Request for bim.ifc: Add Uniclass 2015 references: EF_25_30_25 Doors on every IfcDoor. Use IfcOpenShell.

First a look at what the model holds.

```python
import ifcopenshell

model = ifcopenshell.open("bim.ifc")
print(model.schema)
print("classifications:", [c.Name for c in model.by_type("IfcClassification")])
for ifc_class in ("IfcDoor", "IfcRoof", "IfcStair", "IfcWall", "IfcWindow"):
    print(ifc_class, len(model.by_type(ifc_class)))
```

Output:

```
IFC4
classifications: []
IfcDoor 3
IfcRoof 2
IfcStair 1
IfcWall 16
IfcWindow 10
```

```python
import ifcopenshell
import ifcopenshell.api.classification

model = ifcopenshell.open("bim.ifc")

system = ifcopenshell.api.classification.add_classification(model, classification="Uniclass 2015")

codes = {
    "IfcDoor": ("EF_25_30_25", "Doors"),
}
for ifc_class, (code, name) in codes.items():
    products = model.by_type(ifc_class)
    ifcopenshell.api.classification.add_reference(
        model, products=products, classification=system, identification=code, name=name
    )
    print(code, len(products))

model.write("bim_updated.ifc")
```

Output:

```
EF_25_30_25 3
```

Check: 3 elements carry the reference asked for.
